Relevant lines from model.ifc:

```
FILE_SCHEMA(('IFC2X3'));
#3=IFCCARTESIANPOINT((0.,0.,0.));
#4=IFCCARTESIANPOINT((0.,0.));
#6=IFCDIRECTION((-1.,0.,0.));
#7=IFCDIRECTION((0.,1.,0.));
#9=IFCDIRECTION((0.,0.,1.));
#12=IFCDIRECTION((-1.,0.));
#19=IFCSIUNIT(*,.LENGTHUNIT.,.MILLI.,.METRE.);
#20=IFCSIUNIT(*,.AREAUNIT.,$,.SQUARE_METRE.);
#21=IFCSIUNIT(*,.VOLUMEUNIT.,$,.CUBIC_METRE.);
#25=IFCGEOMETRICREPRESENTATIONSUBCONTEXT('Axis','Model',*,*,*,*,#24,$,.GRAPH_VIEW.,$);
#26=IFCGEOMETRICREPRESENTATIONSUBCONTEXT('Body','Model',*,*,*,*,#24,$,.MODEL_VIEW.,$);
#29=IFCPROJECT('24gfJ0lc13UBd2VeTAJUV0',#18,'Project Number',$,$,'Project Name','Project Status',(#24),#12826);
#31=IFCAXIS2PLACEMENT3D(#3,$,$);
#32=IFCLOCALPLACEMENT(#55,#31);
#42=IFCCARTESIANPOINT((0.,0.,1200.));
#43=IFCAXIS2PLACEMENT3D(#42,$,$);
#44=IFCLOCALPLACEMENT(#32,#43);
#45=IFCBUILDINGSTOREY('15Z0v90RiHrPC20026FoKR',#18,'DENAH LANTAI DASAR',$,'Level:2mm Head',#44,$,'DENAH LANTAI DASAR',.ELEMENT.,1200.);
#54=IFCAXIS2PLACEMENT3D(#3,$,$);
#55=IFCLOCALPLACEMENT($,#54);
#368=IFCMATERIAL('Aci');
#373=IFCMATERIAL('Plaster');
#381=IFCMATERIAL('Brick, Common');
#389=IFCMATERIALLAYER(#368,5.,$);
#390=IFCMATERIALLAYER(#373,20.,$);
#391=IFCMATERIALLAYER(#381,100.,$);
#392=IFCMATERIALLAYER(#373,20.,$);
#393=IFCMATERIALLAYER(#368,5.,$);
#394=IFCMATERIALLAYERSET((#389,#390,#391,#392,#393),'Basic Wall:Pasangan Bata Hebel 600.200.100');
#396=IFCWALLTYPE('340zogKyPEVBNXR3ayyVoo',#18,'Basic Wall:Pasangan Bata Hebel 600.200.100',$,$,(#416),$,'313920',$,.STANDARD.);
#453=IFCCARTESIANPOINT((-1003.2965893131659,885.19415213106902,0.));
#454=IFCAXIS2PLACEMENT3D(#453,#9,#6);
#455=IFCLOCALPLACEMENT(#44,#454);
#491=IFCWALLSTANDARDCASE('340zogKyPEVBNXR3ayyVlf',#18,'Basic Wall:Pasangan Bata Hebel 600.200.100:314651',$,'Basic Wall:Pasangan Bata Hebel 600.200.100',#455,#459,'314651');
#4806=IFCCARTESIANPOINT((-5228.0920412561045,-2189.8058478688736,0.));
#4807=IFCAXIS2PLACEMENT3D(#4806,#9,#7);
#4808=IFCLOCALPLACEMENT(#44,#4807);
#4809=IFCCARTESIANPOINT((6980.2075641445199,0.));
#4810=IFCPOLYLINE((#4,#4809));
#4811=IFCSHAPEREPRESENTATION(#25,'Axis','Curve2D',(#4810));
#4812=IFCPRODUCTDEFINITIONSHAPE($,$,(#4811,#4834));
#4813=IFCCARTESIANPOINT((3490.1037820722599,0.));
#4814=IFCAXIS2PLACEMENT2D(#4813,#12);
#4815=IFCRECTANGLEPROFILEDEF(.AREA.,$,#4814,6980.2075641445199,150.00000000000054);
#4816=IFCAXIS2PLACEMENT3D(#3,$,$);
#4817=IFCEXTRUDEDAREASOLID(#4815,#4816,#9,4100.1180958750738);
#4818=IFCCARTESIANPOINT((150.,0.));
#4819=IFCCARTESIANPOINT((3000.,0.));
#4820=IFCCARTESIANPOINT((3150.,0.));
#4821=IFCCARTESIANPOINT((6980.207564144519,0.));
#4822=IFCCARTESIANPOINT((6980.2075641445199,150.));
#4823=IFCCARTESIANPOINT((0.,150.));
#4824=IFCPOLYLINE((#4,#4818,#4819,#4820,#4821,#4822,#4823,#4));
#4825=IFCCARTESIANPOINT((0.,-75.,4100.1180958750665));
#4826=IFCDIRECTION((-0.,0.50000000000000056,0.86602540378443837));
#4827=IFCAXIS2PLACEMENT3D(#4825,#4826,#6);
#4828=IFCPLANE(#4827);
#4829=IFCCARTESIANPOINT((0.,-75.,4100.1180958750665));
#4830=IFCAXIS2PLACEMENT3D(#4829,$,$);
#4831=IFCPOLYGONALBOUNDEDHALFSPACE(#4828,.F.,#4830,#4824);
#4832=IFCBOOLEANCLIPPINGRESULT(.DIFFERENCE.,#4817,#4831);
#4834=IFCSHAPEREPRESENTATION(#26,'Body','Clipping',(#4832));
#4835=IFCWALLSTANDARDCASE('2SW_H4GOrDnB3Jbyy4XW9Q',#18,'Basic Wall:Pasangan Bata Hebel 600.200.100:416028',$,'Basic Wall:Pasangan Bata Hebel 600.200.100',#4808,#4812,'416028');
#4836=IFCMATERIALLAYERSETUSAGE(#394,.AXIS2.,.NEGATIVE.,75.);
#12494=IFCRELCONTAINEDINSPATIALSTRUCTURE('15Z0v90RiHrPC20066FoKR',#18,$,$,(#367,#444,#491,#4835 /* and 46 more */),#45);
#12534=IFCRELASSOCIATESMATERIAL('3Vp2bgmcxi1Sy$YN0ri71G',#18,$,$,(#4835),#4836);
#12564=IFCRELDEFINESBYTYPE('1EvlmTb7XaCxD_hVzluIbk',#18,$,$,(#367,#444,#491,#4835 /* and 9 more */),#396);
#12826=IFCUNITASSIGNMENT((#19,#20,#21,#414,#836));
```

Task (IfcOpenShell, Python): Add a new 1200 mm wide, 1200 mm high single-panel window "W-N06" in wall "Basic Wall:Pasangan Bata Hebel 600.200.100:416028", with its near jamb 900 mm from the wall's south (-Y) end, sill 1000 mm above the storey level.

```python
import numpy as np
import ifcopenshell
import ifcopenshell.api.feature
import ifcopenshell.api.geometry
import ifcopenshell.api.root
import ifcopenshell.api.spatial
import ifcopenshell.api.type
import ifcopenshell.geom
import ifcopenshell.util.element
import ifcopenshell.util.placement
import ifcopenshell.util.representation
import ifcopenshell.util.shape
import ifcopenshell.util.unit

model = ifcopenshell.open("model.ifc")
unit_scale = ifcopenshell.util.unit.calculate_unit_scale(model)
settings = ifcopenshell.geom.settings()


def volume(element):
    """Net volume in cubic metres, openings subtracted."""
    shape = ifcopenshell.geom.create_shape(settings, element)
    return ifcopenshell.util.shape.get_volume(shape.geometry)


wall = model.by_id(4835)
storey = ifcopenshell.util.element.get_container(wall, ifc_class="IfcBuildingStorey")
context = ifcopenshell.util.representation.get_context(model, "Model", "Body", "MODEL_VIEW")
before = volume(wall)

width, height, from_end, sill = 1.2, 1.2, 0.9, 1  # metres

# The wall runs along its own X axis, and the end named is its -X end.
wall_shape = ifcopenshell.geom.create_shape(settings, wall)
x, y, z = ifcopenshell.util.shape.get_vertices(wall_shape.geometry).T
start = x.min() + from_end
face, thickness = float(y.min()), float(y.max() - y.min())
wall_matrix = ifcopenshell.util.placement.get_local_placement(wall.ObjectPlacement)
level = ifcopenshell.util.placement.get_local_placement(storey.ObjectPlacement)[2, 3]


def in_wall(x, y):
    """Placement at x, y metres in the wall's axes, at sill height."""
    matrix = wall_matrix.copy()
    matrix[:, 3] = wall_matrix @ np.array([x / unit_scale, y / unit_scale, 0.0, 1.0])
    matrix[2, 3] = level + sill / unit_scale
    return matrix


# Opening: a box that overshoots both wall faces by 50 mm.
opening = ifcopenshell.api.root.create_entity(model, ifc_class="IfcOpeningElement")
box = ifcopenshell.api.geometry.add_wall_representation(
    model, context=context, length=width, height=height, thickness=thickness + 0.1
)
ifcopenshell.api.geometry.assign_representation(model, product=opening, representation=box)
ifcopenshell.api.geometry.edit_object_placement(model, product=opening, matrix=in_wall(start, face - 0.05), is_si=False)
ifcopenshell.api.feature.add_feature(model, feature=opening, element=wall)

window = ifcopenshell.api.root.create_entity(model, ifc_class="IfcWindow", name="W-N06")
window.OverallWidth, window.OverallHeight = width / unit_scale, height / unit_scale
body = ifcopenshell.api.geometry.add_window_representation(
    model,
    context=context,
    overall_width=window.OverallWidth,
    overall_height=window.OverallHeight,
    partition_type="SINGLE_PANEL",
)
ifcopenshell.api.geometry.assign_representation(model, product=window, representation=body)
ifcopenshell.api.spatial.assign_container(model, products=[window], relating_structure=storey)
fills = ifcopenshell.api.feature.add_filling(model, opening=opening, element=window)
fills.OwnerHistory = window.OwnerHistory  # required in IFC2X3

# IFC2X3 keeps the operation on the window style.
style = ifcopenshell.api.root.create_entity(model, ifc_class="IfcWindowStyle", name="W-N06")
style.OperationType, style.ConstructionType = "SINGLE_PANEL", "NOTDEFINED"
style.ParameterTakesPrecedence = style.Sizeable = False
ifcopenshell.api.type.assign_type(model, related_objects=[window], relating_type=style)

# Centre the window in the wall's thickness.
ifcopenshell.api.geometry.edit_object_placement(model, product=window, matrix=in_wall(start, face), is_si=False)
window_shape = ifcopenshell.geom.create_shape(settings, window)
depth = ifcopenshell.util.shape.get_vertices(window_shape.geometry)[:, 1]
offset = face + thickness / 2 - (depth.min() + depth.max()) / 2
ifcopenshell.api.geometry.edit_object_placement(model, product=window, matrix=in_wall(start, offset), is_si=False)

after = volume(wall)

print(f"wall volume {before:.3f} -> {after:.3f} m3")

model.write("model_updated.ifc")
```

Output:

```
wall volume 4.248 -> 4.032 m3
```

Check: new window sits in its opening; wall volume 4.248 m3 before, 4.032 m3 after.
